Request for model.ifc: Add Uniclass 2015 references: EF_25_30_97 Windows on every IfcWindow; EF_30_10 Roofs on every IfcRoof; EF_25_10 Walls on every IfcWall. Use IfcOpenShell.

First a look at what the model holds.

```python
import ifcopenshell

model = ifcopenshell.open("model.ifc")
print(model.schema)
print("classifications:", [c.Name for c in model.by_type("IfcClassification")])
for ifc_class in ("IfcDoor", "IfcRoof", "IfcStair", "IfcWall", "IfcWindow"):
    print(ifc_class, len(model.by_type(ifc_class)))
```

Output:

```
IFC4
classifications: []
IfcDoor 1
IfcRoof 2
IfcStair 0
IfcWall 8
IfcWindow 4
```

```python
import ifcopenshell
import ifcopenshell.api.classification

model = ifcopenshell.open("model.ifc")

system = ifcopenshell.api.classification.add_classification(model, classification="Uniclass 2015")

codes = {
    "IfcWindow": ("EF_25_30_97", "Windows"),
    "IfcRoof": ("EF_30_10", "Roofs"),
    "IfcWall": ("EF_25_10", "Walls"),
}
for ifc_class, (code, name) in codes.items():
    products = model.by_type(ifc_class)
    ifcopenshell.api.classification.add_reference(
        model, products=products, classification=system, identification=code, name=name
    )
    print(code, len(products))

model.write("model-out.ifc")
```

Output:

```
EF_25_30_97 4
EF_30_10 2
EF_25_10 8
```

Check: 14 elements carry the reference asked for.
